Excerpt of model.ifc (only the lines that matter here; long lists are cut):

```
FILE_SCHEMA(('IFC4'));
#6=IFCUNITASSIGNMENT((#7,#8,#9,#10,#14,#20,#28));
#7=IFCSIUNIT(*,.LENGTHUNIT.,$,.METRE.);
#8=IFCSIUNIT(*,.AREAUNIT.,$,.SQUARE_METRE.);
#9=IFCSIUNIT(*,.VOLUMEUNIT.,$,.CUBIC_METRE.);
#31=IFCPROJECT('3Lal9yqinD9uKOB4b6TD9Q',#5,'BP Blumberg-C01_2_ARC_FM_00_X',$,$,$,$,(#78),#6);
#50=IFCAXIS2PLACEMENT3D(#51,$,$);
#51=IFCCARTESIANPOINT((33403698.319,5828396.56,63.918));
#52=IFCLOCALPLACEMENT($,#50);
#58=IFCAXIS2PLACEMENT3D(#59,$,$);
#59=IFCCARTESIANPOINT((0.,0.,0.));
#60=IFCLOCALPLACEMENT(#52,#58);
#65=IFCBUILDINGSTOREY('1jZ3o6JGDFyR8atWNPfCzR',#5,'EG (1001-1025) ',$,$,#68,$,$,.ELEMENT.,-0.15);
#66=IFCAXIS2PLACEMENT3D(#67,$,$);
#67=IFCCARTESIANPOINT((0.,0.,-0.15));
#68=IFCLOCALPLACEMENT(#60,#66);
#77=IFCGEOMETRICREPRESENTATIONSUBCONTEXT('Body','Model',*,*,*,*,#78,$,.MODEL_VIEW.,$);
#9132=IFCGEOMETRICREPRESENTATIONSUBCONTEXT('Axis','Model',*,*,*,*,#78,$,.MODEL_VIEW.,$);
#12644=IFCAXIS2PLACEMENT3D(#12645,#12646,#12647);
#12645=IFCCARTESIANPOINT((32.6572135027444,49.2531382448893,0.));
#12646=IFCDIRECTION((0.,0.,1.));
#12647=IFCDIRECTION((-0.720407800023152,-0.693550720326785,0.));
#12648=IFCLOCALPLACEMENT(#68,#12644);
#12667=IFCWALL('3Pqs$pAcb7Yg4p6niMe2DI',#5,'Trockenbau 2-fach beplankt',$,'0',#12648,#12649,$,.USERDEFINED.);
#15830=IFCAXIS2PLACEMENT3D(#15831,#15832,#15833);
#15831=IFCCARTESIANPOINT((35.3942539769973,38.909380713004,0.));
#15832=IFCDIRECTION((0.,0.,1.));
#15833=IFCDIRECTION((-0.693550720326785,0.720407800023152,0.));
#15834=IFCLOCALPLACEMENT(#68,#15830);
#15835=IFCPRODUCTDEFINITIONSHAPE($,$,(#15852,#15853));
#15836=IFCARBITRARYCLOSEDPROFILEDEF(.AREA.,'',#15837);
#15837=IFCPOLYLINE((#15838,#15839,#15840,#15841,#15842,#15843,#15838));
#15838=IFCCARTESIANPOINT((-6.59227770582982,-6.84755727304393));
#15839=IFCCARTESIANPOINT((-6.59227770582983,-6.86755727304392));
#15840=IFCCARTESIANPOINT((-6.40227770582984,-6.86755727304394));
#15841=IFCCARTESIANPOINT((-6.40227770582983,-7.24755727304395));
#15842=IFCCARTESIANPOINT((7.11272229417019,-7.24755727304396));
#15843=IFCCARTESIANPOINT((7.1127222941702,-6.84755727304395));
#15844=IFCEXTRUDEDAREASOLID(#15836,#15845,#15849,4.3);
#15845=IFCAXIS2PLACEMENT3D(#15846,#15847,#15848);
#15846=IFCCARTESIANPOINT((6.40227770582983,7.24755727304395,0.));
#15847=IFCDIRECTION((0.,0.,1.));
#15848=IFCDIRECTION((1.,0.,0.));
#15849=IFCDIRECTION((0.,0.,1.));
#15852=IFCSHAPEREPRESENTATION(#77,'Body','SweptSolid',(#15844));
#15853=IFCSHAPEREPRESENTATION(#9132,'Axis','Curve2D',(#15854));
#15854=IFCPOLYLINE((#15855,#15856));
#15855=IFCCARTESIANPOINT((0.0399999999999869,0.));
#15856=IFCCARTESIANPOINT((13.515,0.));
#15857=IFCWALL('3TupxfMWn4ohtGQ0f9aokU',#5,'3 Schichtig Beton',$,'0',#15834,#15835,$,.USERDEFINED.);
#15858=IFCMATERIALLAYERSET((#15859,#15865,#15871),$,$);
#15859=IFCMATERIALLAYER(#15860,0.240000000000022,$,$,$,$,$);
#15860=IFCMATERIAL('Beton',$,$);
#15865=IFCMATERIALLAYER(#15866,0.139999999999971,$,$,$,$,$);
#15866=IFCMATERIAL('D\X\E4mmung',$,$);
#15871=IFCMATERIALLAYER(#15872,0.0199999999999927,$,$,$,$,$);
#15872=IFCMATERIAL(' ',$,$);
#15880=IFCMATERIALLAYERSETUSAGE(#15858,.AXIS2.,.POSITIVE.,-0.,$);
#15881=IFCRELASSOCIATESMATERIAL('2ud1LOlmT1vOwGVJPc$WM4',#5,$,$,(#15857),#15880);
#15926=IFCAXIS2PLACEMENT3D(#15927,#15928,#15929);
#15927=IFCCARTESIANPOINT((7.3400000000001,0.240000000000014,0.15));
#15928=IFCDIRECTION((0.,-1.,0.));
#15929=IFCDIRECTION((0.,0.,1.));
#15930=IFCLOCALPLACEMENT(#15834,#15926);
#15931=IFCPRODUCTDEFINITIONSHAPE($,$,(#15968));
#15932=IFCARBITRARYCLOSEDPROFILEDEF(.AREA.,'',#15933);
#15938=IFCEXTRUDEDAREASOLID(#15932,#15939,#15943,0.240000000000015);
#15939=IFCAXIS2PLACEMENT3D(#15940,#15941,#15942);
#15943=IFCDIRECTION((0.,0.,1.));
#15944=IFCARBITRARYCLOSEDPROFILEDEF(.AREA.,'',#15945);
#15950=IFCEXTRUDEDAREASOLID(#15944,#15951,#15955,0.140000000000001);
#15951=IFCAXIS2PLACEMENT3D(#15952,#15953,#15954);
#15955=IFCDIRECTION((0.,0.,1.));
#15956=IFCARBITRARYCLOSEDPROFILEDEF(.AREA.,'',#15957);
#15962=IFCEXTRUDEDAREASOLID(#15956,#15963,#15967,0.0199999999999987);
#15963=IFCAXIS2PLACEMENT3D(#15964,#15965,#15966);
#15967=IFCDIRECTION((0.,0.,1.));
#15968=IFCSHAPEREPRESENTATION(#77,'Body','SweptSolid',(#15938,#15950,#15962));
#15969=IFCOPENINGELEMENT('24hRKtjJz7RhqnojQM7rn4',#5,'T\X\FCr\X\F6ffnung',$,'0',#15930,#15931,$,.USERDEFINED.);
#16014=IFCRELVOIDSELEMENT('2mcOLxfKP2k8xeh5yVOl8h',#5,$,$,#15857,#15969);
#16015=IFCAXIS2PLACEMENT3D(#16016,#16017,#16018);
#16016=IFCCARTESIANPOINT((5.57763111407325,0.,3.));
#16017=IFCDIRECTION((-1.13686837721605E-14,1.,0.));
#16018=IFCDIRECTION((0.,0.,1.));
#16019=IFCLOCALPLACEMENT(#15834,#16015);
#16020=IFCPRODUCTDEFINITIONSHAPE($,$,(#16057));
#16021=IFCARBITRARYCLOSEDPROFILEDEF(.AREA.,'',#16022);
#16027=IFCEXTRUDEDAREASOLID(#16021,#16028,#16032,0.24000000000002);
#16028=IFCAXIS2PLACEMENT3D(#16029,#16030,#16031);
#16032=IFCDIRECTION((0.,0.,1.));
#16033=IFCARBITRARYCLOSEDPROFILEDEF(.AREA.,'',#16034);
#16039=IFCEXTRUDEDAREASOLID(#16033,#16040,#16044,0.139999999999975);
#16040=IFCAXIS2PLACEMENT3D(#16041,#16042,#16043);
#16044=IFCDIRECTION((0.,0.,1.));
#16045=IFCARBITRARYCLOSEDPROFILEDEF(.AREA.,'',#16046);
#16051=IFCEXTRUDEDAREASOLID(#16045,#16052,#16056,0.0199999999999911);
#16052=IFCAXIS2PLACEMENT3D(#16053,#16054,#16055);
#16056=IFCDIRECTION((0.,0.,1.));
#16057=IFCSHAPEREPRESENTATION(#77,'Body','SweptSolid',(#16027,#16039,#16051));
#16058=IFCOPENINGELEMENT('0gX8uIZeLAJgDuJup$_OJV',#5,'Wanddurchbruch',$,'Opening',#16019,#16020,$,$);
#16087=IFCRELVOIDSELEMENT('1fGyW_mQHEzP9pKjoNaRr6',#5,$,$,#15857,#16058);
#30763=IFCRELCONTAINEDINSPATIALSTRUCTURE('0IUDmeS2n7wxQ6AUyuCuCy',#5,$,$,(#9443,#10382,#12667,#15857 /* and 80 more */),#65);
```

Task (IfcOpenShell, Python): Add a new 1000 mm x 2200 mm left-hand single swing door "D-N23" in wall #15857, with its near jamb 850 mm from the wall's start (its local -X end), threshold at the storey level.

```python
import numpy as np
import ifcopenshell
import ifcopenshell.api.feature
import ifcopenshell.api.geometry
import ifcopenshell.api.root
import ifcopenshell.api.spatial
import ifcopenshell.geom
import ifcopenshell.util.element
import ifcopenshell.util.placement
import ifcopenshell.util.representation
import ifcopenshell.util.shape
import ifcopenshell.util.unit

model = ifcopenshell.open("model.ifc")
unit_scale = ifcopenshell.util.unit.calculate_unit_scale(model)
settings = ifcopenshell.geom.settings()


def volume(element):
    """Net volume in cubic metres, openings subtracted."""
    shape = ifcopenshell.geom.create_shape(settings, element)
    return ifcopenshell.util.shape.get_volume(shape.geometry)


wall = model.by_id(15857)
storey = ifcopenshell.util.element.get_container(wall, ifc_class="IfcBuildingStorey")
context = ifcopenshell.util.representation.get_context(model, "Model", "Body", "MODEL_VIEW")
before = volume(wall)

width, height, from_end, sill = 1, 2.2, 0.85, 0.0  # metres

# The wall runs along its own X axis, and the end named is its -X end.
wall_shape = ifcopenshell.geom.create_shape(settings, wall)
x, y, z = ifcopenshell.util.shape.get_vertices(wall_shape.geometry).T
start = x.min() + from_end
face, thickness = float(y.min()), float(y.max() - y.min())
wall_matrix = ifcopenshell.util.placement.get_local_placement(wall.ObjectPlacement)
level = ifcopenshell.util.placement.get_local_placement(storey.ObjectPlacement)[2, 3]


def in_wall(x, y):
    """Placement at x, y metres in the wall's axes, at sill height."""
    matrix = wall_matrix.copy()
    matrix[:, 3] = wall_matrix @ np.array([x / unit_scale, y / unit_scale, 0.0, 1.0])
    matrix[2, 3] = level + sill / unit_scale
    return matrix


# Opening: a box that overshoots both wall faces by 50 mm.
opening = ifcopenshell.api.root.create_entity(model, ifc_class="IfcOpeningElement", predefined_type="OPENING")
box = ifcopenshell.api.geometry.add_wall_representation(
    model, context=context, length=width, height=height, thickness=thickness + 0.1
)
ifcopenshell.api.geometry.assign_representation(model, product=opening, representation=box)
ifcopenshell.api.geometry.edit_object_placement(model, product=opening, matrix=in_wall(start, face - 0.05), is_si=False)
ifcopenshell.api.feature.add_feature(model, feature=opening, element=wall)

door = ifcopenshell.api.root.create_entity(model, ifc_class="IfcDoor", name="D-N23", predefined_type="DOOR")
door.OverallWidth, door.OverallHeight = width / unit_scale, height / unit_scale
door.OperationType = "SINGLE_SWING_LEFT"
body = ifcopenshell.api.geometry.add_door_representation(
    model,
    context=context,
    overall_width=door.OverallWidth,
    overall_height=door.OverallHeight,
    operation_type="SINGLE_SWING_LEFT",
    lining_properties={"LiningDepth": thickness / unit_scale, "ThresholdDepth": thickness / unit_scale},
)
ifcopenshell.api.geometry.assign_representation(model, product=door, representation=body)
ifcopenshell.api.spatial.assign_container(model, products=[door], relating_structure=storey)
ifcopenshell.api.feature.add_filling(model, opening=opening, element=door)

# The lining spans the wall, so the door starts at the wall face.
ifcopenshell.api.geometry.edit_object_placement(model, product=door, matrix=in_wall(start, face), is_si=False)

after = volume(wall)

print(f"wall volume {before:.3f} -> {after:.3f} m3")

model.write("model_edited.ifc")
```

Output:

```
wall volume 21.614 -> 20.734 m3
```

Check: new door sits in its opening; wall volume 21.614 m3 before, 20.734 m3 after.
